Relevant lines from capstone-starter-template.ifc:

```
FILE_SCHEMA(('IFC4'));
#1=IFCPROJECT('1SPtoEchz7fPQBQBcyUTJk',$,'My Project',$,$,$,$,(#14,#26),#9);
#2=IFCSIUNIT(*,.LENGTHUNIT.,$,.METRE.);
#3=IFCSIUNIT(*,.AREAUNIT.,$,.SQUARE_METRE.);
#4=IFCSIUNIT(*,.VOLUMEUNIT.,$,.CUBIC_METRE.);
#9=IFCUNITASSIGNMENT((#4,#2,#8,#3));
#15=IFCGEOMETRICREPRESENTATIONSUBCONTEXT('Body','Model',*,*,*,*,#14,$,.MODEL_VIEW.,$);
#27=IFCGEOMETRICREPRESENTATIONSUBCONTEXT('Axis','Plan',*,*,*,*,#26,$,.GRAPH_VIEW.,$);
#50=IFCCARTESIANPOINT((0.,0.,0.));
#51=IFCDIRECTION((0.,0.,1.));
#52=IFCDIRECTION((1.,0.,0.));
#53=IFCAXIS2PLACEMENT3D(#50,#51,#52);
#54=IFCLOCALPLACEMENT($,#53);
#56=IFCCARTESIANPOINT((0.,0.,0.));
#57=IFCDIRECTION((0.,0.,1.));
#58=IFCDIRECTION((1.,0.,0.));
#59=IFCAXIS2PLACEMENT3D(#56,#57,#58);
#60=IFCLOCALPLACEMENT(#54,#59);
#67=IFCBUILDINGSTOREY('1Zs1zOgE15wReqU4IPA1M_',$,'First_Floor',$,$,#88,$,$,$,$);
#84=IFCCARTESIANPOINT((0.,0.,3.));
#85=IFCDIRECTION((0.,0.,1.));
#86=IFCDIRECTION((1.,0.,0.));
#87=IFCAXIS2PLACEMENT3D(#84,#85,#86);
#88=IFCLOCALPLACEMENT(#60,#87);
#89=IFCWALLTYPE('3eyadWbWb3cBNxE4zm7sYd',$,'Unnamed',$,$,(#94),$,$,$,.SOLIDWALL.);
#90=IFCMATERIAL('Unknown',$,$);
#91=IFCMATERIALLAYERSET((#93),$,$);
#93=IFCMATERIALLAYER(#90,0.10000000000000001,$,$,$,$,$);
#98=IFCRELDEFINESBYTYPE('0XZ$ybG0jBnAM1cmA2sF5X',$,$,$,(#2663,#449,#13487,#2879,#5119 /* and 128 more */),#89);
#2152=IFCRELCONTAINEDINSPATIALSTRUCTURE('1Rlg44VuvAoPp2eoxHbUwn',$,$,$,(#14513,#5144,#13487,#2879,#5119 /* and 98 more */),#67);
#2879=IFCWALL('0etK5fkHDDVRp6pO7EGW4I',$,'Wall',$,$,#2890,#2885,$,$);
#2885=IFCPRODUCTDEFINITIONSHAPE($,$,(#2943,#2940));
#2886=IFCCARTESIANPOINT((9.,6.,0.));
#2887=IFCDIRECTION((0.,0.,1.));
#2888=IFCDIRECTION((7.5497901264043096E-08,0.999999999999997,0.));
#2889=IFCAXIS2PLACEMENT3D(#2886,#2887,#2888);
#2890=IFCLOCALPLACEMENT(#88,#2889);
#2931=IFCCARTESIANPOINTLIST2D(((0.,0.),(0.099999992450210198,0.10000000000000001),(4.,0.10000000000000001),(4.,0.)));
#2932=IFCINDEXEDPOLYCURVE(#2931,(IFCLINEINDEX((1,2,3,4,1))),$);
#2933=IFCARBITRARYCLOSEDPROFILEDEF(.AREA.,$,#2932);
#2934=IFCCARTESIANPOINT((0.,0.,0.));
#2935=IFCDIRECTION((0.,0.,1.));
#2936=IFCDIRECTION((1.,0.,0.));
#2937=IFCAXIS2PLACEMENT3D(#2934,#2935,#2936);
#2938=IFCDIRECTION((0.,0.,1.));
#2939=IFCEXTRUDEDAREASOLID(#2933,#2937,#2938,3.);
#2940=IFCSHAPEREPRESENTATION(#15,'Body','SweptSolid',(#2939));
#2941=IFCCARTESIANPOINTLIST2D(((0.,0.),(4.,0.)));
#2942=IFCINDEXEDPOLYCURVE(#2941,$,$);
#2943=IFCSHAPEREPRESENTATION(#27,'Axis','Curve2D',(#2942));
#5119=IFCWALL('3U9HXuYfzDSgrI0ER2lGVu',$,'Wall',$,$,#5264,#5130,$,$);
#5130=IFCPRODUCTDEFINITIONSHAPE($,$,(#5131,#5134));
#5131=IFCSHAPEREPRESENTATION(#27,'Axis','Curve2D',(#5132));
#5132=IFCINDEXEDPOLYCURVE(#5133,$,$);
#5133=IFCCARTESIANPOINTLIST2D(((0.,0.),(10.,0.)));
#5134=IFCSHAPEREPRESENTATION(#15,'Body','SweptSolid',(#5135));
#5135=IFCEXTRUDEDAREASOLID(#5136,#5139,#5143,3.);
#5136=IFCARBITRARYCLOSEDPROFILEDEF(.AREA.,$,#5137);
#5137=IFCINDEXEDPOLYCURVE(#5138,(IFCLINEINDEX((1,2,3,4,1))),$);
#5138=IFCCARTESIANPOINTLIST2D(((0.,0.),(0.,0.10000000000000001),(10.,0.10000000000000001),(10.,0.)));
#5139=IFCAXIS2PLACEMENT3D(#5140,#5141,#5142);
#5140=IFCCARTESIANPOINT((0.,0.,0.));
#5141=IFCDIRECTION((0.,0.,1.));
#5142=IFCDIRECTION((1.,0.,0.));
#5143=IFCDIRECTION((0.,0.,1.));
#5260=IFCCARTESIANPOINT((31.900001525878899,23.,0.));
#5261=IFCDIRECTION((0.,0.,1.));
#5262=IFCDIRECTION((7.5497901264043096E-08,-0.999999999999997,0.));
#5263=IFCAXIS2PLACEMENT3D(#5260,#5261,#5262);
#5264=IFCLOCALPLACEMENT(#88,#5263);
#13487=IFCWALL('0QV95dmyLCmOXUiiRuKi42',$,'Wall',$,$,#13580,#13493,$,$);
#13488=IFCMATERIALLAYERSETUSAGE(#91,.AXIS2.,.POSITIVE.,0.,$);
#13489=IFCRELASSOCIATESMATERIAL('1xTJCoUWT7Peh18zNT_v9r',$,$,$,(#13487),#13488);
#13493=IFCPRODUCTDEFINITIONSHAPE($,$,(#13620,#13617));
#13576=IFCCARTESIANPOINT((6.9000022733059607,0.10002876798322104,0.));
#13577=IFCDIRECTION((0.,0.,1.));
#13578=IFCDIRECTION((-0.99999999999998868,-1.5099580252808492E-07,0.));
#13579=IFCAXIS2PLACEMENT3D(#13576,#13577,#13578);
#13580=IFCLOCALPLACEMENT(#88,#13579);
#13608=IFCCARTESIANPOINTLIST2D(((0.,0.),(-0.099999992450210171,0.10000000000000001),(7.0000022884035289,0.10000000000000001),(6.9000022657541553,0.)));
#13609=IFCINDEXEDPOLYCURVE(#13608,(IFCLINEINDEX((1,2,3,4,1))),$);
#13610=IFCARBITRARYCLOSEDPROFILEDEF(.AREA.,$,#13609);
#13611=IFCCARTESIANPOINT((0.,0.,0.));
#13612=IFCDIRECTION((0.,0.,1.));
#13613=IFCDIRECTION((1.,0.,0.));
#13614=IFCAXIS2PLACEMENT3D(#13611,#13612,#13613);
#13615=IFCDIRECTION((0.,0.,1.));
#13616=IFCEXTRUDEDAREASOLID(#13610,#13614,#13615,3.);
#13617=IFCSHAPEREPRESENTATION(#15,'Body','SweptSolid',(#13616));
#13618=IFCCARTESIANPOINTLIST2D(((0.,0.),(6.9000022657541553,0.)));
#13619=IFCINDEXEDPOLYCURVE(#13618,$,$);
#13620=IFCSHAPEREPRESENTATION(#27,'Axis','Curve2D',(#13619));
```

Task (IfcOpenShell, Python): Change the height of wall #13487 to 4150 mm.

```python
import ifcopenshell
import ifcopenshell.geom
import ifcopenshell.util.representation
import ifcopenshell.util.shape
import ifcopenshell.util.unit

model = ifcopenshell.open("capstone-starter-template.ifc")
unit_scale = ifcopenshell.util.unit.calculate_unit_scale(model)
settings = ifcopenshell.geom.settings()


def volume(element):
    """Net volume in cubic metres, openings subtracted."""
    shape = ifcopenshell.geom.create_shape(settings, element)
    return ifcopenshell.util.shape.get_volume(shape.geometry)


wall = model.by_guid("0QV95dmyLCmOXUiiRuKi42")
before = volume(wall)

body = ifcopenshell.util.representation.get_representation(wall, "Model", "Body")
solid = body.Items[0]
old_height = solid.Depth
solid.Depth = 4.15 / unit_scale
after = volume(wall)

print(f"height {old_height:g} -> {solid.Depth:g}, volume {before:.3f} -> {after:.3f} m3")

model.write("capstone-starter-template-out.ifc")
```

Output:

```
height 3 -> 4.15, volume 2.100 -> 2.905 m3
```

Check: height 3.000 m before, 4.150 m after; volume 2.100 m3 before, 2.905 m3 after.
